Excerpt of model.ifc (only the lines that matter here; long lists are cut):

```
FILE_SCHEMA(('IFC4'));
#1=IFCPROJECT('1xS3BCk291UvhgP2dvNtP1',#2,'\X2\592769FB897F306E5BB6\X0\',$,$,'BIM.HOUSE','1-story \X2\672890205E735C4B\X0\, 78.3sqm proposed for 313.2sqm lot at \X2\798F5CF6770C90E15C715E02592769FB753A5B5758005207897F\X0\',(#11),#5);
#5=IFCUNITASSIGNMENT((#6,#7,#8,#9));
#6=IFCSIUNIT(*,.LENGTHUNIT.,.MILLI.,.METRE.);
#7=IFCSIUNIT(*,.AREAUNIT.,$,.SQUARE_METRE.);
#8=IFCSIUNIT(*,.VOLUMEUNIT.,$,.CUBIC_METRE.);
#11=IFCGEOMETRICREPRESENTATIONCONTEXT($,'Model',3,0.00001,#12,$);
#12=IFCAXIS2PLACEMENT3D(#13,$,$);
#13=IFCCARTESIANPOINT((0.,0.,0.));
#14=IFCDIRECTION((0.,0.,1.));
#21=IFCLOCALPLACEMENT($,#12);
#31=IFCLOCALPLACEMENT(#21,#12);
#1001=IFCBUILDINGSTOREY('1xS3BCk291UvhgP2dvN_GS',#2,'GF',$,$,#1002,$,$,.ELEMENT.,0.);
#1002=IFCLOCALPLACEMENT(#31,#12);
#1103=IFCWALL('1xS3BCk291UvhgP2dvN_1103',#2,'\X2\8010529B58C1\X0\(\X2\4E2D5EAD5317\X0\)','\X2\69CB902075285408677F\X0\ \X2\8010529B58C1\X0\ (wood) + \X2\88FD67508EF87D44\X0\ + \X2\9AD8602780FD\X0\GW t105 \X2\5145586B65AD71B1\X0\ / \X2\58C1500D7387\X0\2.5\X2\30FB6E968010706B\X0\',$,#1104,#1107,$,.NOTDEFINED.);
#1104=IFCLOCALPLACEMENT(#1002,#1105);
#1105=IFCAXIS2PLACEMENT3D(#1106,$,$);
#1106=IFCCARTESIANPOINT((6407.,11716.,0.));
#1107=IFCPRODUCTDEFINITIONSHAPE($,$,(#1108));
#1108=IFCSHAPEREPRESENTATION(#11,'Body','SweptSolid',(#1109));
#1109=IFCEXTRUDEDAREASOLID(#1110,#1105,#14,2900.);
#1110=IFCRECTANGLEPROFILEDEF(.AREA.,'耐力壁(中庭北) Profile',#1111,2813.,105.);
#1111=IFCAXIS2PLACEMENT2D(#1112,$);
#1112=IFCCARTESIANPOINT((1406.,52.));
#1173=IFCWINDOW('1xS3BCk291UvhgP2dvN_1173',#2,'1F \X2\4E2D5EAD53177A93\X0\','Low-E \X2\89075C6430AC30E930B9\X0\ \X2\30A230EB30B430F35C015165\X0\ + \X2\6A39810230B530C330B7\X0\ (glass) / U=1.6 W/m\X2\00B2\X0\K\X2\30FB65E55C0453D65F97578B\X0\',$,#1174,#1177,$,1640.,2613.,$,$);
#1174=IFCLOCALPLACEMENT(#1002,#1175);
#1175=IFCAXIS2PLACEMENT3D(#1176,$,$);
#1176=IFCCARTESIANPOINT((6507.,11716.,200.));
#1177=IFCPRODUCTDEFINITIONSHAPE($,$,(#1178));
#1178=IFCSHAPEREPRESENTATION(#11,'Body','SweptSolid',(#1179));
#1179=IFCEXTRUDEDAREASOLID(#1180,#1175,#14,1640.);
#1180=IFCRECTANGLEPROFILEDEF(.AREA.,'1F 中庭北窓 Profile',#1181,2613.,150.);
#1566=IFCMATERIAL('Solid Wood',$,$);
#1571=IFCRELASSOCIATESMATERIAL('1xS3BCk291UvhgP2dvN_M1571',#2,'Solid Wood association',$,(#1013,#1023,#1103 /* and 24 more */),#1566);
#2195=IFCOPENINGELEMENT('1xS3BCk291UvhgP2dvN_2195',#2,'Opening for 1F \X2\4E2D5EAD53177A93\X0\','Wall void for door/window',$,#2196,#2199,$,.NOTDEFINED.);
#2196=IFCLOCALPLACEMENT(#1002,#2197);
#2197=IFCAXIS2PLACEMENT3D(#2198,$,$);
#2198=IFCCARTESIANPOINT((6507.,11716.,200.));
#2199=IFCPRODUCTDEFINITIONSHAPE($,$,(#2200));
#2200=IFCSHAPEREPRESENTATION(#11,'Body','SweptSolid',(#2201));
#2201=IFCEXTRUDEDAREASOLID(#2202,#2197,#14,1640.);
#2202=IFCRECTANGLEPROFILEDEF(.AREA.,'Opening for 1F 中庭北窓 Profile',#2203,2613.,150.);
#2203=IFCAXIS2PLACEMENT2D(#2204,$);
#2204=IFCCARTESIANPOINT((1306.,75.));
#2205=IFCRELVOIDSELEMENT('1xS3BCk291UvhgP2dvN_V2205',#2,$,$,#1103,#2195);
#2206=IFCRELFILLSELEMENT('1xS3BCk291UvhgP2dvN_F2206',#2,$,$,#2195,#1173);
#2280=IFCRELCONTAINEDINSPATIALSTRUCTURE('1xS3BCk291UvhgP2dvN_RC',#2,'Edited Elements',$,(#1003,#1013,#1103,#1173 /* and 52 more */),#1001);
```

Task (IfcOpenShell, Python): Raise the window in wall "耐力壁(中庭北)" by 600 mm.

```python
import numpy as np
import ifcopenshell
import ifcopenshell.api.geometry
import ifcopenshell.util.placement
import ifcopenshell.util.unit

model = ifcopenshell.open("model.ifc")
unit_scale = ifcopenshell.util.unit.calculate_unit_scale(model)

window = model.by_guid("1xS3BCk291UvhgP2dvN_1173")
opening = window.FillsVoids[0].RelatingOpeningElement
dz = 600.0

shift = np.array([0.0, 0.0, dz])
# The window is not placed relative to its opening, so move both.
for product in (opening, window):
    matrix = ifcopenshell.util.placement.get_local_placement(product.ObjectPlacement)
    matrix[:3, 3] += shift
    ifcopenshell.api.geometry.edit_object_placement(model, product=product, matrix=matrix, is_si=False)

print(f"moved by {dz * unit_scale:+.3f} m")

model.write("model_edited.ifc")
```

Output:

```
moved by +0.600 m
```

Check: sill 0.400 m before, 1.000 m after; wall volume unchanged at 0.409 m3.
